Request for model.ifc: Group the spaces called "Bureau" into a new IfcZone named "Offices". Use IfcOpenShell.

First a look at what the model holds.

```python
import ifcopenshell

model = ifcopenshell.open("model.ifc")
print(model.schema)
seen = {}
for space in model.by_type("IfcSpace"):
    seen[space.LongName] = seen.get(space.LongName, 0) + 1
for name, count in sorted(seen.items(), key=str):
    print(count, "x", name)
print("zones:", [z.Name for z in model.by_type("IfcZone")][:20])
```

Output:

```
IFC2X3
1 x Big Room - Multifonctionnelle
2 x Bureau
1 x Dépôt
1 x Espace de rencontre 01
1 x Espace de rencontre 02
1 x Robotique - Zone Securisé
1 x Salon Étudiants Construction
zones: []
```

```python
import ifcopenshell
import ifcopenshell.api.group
import ifcopenshell.api.root

model = ifcopenshell.open("model.ifc")

names = {"Bureau"}
spaces = [s for s in model.by_type("IfcSpace") if s.LongName in names]

zone = ifcopenshell.api.root.create_entity(model, ifc_class="IfcZone", name="Offices")
ifcopenshell.api.group.assign_group(model, products=spaces, group=zone)
print(len(spaces), "spaces in", zone.Name)

model.write("model_edited.ifc")
```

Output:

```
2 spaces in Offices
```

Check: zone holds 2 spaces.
